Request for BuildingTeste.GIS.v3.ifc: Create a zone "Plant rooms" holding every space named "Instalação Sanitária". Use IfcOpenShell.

First a look at what the model holds.

```python
import ifcopenshell

model = ifcopenshell.open("BuildingTeste.GIS.v3.ifc")
print(model.schema)
seen = {}
for space in model.by_type("IfcSpace"):
    seen[space.LongName] = seen.get(space.LongName, 0) + 1
for name, count in sorted(seen.items(), key=str):
    print(count, "x", name)
print("zones:", [z.Name for z in model.by_type("IfcZone")][:20])
```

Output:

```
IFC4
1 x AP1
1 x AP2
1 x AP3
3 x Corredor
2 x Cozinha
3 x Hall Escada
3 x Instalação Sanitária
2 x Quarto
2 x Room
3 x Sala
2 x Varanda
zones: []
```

```python
import ifcopenshell
import ifcopenshell.api.group
import ifcopenshell.api.root

model = ifcopenshell.open("BuildingTeste.GIS.v3.ifc")

names = {"Instalação Sanitária"}
spaces = [s for s in model.by_type("IfcSpace") if s.LongName in names]

zone = ifcopenshell.api.root.create_entity(model, ifc_class="IfcZone", name="Plant rooms")
ifcopenshell.api.group.assign_group(model, products=spaces, group=zone)
print(len(spaces), "spaces in", zone.Name)

model.write("BuildingTeste.GIS.v3_updated.ifc")
```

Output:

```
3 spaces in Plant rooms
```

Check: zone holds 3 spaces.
